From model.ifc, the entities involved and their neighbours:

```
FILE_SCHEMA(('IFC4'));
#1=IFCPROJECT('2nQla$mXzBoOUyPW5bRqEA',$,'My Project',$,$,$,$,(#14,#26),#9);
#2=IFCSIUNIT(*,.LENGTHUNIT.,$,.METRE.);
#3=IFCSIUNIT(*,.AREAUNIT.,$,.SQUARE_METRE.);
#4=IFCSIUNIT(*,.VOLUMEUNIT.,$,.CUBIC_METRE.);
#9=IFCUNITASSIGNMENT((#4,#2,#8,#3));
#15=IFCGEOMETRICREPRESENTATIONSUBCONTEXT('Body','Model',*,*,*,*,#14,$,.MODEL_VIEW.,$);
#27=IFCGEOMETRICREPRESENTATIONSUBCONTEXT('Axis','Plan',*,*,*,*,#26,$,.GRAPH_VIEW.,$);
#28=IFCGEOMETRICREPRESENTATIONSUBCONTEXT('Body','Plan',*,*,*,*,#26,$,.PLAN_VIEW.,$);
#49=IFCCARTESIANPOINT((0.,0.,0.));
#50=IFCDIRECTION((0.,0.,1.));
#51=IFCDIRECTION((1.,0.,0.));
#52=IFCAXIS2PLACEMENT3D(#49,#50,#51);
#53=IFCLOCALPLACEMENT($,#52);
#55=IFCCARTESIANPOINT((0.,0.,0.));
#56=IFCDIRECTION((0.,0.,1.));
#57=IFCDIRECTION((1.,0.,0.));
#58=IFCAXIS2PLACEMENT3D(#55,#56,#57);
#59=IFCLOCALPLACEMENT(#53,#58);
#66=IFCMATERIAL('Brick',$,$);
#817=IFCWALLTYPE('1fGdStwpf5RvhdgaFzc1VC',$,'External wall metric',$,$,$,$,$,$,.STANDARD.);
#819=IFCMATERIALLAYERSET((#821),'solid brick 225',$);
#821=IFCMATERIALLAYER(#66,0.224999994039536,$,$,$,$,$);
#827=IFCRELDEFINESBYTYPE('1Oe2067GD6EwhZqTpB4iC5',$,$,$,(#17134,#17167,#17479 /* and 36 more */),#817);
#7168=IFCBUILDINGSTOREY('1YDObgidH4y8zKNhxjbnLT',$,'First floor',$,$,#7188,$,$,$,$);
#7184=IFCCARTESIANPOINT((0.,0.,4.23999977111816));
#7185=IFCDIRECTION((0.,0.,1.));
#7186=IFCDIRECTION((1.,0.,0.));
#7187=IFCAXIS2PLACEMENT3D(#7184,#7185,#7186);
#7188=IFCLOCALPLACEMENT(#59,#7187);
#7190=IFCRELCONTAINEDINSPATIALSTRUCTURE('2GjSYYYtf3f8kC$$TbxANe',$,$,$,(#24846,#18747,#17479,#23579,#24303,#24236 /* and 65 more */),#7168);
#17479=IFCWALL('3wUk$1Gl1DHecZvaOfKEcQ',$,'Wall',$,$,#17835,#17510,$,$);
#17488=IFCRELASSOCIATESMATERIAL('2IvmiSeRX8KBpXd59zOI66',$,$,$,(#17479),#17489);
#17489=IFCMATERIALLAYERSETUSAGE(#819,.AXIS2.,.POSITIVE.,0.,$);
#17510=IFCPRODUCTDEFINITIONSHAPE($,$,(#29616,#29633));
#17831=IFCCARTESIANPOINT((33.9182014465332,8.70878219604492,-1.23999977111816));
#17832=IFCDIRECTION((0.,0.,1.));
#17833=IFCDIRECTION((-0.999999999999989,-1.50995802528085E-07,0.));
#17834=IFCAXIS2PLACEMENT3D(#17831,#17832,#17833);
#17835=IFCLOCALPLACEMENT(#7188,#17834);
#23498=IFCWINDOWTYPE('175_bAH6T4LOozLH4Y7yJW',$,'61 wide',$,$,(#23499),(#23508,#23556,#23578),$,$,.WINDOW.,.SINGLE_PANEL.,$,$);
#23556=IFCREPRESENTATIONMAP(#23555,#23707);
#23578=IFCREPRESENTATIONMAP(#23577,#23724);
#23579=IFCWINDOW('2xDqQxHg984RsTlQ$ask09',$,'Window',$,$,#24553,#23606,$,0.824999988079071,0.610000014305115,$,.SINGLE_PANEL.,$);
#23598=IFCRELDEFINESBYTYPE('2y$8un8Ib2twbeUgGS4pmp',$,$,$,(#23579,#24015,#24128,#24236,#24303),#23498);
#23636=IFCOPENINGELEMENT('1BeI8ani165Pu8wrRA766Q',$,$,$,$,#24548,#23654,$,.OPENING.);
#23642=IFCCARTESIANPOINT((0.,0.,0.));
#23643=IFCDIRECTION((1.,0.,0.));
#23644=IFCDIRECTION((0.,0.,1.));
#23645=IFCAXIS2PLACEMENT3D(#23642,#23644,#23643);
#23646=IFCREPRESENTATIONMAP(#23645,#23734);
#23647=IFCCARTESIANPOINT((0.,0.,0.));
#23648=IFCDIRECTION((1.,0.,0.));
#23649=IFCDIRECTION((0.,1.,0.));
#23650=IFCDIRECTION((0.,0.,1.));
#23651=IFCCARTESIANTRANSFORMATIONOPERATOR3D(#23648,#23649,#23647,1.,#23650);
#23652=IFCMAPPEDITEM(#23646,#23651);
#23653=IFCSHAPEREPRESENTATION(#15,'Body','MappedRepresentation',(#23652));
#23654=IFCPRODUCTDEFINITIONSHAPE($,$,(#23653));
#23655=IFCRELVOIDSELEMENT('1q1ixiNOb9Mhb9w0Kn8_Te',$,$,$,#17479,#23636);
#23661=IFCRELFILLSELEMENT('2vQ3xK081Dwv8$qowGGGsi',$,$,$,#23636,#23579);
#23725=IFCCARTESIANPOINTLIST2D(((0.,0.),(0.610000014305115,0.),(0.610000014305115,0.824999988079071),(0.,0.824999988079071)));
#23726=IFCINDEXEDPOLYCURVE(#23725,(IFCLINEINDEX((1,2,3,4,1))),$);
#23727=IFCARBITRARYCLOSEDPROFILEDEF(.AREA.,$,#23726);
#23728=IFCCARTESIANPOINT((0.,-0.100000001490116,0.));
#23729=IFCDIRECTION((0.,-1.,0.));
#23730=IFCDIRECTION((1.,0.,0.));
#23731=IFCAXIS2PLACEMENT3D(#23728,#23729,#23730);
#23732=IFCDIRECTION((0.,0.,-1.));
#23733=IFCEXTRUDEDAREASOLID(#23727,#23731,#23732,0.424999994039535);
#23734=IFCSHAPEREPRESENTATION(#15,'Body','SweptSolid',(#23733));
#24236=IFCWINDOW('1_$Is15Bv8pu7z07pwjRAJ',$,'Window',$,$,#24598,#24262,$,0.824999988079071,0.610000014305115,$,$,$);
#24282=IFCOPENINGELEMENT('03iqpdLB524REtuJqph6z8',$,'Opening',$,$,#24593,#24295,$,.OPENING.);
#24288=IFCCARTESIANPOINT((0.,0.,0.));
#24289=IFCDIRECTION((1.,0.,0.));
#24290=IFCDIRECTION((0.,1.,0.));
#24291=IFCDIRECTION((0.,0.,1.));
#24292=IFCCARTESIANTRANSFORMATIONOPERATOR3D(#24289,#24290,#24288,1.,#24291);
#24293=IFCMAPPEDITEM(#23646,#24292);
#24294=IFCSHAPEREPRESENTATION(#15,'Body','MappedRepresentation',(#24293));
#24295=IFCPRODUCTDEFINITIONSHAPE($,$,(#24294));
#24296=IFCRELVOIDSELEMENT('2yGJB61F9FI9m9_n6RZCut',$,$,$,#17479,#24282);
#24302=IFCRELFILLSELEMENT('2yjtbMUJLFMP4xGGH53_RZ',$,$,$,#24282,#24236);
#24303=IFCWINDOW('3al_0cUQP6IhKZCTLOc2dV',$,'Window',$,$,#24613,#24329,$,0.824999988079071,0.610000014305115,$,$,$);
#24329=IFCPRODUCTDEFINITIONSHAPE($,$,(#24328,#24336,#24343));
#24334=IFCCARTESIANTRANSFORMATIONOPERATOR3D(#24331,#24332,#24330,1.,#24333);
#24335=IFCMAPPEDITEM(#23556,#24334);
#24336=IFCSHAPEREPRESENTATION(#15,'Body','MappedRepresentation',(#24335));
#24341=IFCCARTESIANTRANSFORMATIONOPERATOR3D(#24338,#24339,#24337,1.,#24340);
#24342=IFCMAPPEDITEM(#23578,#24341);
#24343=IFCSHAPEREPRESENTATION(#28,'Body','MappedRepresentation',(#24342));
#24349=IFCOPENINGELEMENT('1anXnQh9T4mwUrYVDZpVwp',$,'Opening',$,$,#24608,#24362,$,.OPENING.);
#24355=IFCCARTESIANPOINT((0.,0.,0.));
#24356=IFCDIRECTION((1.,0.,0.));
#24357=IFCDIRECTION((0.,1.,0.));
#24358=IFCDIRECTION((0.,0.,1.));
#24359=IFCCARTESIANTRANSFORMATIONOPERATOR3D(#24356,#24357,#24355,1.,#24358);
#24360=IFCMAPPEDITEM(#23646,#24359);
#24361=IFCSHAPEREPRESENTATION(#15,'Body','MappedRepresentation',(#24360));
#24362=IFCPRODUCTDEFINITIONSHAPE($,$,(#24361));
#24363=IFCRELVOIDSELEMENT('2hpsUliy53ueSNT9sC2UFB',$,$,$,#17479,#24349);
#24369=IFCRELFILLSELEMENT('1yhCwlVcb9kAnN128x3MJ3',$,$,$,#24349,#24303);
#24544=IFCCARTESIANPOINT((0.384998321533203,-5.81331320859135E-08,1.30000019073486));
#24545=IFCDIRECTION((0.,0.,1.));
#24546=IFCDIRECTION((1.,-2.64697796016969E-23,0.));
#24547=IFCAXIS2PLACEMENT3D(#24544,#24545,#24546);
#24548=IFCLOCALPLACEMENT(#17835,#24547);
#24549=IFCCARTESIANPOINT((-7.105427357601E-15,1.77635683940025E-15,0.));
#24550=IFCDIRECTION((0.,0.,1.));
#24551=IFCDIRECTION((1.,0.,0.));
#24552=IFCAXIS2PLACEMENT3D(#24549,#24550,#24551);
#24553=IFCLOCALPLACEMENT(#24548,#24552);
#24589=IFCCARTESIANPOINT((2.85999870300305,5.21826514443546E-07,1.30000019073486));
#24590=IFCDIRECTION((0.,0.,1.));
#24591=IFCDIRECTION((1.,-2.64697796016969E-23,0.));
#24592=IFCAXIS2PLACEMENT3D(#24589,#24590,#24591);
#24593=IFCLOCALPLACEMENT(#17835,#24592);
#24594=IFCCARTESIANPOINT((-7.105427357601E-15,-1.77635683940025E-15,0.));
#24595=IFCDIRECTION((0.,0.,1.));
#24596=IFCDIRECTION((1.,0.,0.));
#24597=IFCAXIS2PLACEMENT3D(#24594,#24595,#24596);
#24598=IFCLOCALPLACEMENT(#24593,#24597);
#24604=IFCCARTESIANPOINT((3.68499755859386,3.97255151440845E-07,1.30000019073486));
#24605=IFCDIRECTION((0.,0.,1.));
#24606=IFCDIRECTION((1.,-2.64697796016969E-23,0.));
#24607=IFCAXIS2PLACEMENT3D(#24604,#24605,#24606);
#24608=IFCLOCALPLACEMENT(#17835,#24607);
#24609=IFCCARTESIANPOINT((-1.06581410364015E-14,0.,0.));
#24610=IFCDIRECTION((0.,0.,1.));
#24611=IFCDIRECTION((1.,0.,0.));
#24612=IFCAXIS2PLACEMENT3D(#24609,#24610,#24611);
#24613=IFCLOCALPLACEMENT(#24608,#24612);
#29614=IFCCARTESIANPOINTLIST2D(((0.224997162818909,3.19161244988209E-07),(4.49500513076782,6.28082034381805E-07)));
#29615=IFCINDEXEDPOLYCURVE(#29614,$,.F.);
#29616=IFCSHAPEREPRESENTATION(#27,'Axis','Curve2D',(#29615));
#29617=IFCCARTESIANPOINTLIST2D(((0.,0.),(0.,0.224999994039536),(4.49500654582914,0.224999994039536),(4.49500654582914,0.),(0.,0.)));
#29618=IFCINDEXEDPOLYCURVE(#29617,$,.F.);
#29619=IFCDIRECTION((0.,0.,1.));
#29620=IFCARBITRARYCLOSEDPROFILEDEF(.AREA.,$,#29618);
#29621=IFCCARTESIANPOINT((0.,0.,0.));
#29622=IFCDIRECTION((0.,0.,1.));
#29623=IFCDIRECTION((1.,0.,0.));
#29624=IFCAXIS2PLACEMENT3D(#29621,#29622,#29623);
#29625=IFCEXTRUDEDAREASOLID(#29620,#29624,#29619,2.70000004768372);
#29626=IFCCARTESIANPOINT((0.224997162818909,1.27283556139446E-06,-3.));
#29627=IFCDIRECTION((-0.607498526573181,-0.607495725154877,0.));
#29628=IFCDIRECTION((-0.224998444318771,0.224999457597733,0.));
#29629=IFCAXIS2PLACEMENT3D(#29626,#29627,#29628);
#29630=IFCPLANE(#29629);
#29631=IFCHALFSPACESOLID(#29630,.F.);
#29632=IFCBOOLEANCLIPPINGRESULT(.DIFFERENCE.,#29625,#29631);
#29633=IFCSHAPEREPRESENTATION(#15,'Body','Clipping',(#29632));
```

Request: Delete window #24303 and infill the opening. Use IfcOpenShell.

```python
import ifcopenshell
import ifcopenshell.api.feature
import ifcopenshell.api.root
import ifcopenshell.geom
import ifcopenshell.util.shape

model = ifcopenshell.open("model.ifc")
settings = ifcopenshell.geom.settings()


def volume(element):
    """Net volume in cubic metres, openings subtracted."""
    shape = ifcopenshell.geom.create_shape(settings, element)
    return ifcopenshell.util.shape.get_volume(shape.geometry)


window = model.by_guid("3al_0cUQP6IhKZCTLOc2dV")
opening = window.FillsVoids[0].RelatingOpeningElement
wall = opening.VoidsElements[0].RelatingBuildingElement
before = volume(wall)

ifcopenshell.api.root.remove_product(model, product=window)
ifcopenshell.api.feature.remove_feature(model, feature=opening)

after = volume(wall)

print(f"wall volume {before:.3f} -> {after:.3f} m3")

model.write("model_v2.ifc")
```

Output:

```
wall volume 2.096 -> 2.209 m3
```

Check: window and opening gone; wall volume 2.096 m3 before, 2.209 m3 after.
